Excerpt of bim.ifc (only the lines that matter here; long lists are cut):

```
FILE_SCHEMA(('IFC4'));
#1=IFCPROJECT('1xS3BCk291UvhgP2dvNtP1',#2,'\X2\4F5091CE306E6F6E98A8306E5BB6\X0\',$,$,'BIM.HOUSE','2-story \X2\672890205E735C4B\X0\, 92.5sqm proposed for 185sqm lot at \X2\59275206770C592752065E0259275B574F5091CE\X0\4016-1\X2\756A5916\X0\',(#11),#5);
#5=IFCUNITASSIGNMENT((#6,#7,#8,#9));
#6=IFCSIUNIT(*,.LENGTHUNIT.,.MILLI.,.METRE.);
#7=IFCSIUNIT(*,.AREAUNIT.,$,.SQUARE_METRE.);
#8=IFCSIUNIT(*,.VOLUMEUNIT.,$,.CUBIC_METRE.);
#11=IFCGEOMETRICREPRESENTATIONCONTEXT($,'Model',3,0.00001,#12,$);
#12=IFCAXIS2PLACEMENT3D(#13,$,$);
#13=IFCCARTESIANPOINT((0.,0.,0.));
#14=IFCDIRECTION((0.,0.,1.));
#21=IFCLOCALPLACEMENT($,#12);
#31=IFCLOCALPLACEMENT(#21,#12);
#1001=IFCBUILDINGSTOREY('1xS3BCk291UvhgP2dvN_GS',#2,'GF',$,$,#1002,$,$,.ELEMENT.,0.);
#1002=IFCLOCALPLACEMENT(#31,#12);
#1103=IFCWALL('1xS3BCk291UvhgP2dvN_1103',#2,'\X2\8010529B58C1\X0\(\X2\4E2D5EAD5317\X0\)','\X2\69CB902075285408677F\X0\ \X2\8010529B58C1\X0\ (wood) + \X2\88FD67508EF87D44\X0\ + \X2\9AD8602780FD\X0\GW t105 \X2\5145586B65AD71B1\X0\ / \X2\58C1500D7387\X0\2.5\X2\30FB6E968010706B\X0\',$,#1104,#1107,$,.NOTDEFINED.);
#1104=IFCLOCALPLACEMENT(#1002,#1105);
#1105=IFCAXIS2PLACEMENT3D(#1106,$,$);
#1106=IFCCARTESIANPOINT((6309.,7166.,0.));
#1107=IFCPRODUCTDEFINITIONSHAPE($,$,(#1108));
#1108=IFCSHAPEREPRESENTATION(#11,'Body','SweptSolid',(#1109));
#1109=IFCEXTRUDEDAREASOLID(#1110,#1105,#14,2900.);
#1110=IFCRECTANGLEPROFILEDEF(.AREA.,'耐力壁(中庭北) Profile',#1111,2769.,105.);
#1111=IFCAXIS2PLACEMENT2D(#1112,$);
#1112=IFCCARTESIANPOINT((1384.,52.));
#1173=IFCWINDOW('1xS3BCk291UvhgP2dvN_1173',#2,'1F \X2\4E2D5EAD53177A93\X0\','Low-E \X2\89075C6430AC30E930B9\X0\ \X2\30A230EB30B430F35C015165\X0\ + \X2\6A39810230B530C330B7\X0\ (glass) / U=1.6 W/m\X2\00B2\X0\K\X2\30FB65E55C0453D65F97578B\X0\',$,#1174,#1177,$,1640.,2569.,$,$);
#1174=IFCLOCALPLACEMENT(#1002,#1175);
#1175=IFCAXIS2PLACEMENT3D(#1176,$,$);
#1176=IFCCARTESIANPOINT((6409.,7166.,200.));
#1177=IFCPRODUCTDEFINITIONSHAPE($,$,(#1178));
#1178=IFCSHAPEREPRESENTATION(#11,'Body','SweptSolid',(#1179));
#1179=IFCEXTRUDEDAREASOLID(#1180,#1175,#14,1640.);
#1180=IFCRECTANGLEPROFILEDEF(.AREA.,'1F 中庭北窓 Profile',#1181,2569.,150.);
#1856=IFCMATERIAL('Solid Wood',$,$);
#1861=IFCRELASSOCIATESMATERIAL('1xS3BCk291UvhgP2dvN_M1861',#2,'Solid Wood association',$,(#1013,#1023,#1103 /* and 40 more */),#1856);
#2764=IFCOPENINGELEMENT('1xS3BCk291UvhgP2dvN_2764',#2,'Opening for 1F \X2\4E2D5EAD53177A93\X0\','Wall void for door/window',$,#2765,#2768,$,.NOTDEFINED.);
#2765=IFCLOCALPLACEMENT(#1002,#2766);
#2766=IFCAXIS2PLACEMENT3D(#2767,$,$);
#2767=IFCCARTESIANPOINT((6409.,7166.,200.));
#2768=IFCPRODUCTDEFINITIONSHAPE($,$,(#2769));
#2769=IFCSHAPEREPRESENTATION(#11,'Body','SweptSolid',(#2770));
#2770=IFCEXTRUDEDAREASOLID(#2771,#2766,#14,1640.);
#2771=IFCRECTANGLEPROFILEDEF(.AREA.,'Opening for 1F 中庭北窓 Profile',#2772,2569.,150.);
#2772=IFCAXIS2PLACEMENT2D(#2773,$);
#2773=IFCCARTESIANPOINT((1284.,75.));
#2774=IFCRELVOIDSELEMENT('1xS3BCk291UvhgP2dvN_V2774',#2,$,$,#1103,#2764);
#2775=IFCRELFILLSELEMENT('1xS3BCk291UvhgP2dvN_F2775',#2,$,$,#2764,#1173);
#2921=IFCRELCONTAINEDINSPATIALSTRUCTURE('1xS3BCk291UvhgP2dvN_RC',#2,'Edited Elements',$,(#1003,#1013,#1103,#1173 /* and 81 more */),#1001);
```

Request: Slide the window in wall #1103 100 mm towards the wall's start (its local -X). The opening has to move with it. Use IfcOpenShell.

```python
import ifcopenshell
import ifcopenshell.api.geometry
import ifcopenshell.util.placement
import ifcopenshell.util.unit

model = ifcopenshell.open("bim.ifc")
unit_scale = ifcopenshell.util.unit.calculate_unit_scale(model)

window = model.by_id(1173)
opening = window.FillsVoids[0].RelatingOpeningElement
wall = opening.VoidsElements[0].RelatingBuildingElement

wall_matrix = ifcopenshell.util.placement.get_local_placement(wall.ObjectPlacement)
shift = wall_matrix[:3, 0] * -0.1 / unit_scale
before = ifcopenshell.util.placement.get_local_placement(window.ObjectPlacement)[:3, 3].copy()

# The window is not placed relative to its opening, so move both.
for product in (opening, window):
    matrix = ifcopenshell.util.placement.get_local_placement(product.ObjectPlacement)
    matrix[:3, 3] += shift
    ifcopenshell.api.geometry.edit_object_placement(model, product=product, matrix=matrix, is_si=False)

after = ifcopenshell.util.placement.get_local_placement(window.ObjectPlacement)[:3, 3]
print("window moved by", (after - before).round(3) + 0.0)

model.write("bim_updated.ifc")
```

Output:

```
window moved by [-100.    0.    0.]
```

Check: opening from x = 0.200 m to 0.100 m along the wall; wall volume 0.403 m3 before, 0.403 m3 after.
